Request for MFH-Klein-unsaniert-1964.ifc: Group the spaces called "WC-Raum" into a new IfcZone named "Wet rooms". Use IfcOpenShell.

First a look at what the model holds.

```python
import ifcopenshell

model = ifcopenshell.open("MFH-Klein-unsaniert-1964.ifc")
print(model.schema)
seen = {}
for space in model.by_type("IfcSpace"):
    seen[space.Name] = seen.get(space.Name, 0) + 1
for name, count in sorted(seen.items(), key=str):
    print(count, "x", name)
print("zones:", [z.Name for z in model.by_type("IfcZone")][:20])
```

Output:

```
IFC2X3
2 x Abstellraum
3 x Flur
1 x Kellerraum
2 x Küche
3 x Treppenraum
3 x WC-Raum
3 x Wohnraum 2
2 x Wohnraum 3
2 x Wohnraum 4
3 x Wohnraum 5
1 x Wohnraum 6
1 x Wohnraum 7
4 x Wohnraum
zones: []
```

```python
import ifcopenshell
import ifcopenshell.api.group
import ifcopenshell.api.root

model = ifcopenshell.open("MFH-Klein-unsaniert-1964.ifc")

names = {"WC-Raum"}
spaces = [s for s in model.by_type("IfcSpace") if s.Name in names]

zone = ifcopenshell.api.root.create_entity(model, ifc_class="IfcZone", name="Wet rooms")
ifcopenshell.api.group.assign_group(model, products=spaces, group=zone)
print(len(spaces), "spaces in", zone.Name)

model.write("MFH-Klein-unsaniert-1964_edited.ifc")
```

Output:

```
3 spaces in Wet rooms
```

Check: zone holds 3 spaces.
